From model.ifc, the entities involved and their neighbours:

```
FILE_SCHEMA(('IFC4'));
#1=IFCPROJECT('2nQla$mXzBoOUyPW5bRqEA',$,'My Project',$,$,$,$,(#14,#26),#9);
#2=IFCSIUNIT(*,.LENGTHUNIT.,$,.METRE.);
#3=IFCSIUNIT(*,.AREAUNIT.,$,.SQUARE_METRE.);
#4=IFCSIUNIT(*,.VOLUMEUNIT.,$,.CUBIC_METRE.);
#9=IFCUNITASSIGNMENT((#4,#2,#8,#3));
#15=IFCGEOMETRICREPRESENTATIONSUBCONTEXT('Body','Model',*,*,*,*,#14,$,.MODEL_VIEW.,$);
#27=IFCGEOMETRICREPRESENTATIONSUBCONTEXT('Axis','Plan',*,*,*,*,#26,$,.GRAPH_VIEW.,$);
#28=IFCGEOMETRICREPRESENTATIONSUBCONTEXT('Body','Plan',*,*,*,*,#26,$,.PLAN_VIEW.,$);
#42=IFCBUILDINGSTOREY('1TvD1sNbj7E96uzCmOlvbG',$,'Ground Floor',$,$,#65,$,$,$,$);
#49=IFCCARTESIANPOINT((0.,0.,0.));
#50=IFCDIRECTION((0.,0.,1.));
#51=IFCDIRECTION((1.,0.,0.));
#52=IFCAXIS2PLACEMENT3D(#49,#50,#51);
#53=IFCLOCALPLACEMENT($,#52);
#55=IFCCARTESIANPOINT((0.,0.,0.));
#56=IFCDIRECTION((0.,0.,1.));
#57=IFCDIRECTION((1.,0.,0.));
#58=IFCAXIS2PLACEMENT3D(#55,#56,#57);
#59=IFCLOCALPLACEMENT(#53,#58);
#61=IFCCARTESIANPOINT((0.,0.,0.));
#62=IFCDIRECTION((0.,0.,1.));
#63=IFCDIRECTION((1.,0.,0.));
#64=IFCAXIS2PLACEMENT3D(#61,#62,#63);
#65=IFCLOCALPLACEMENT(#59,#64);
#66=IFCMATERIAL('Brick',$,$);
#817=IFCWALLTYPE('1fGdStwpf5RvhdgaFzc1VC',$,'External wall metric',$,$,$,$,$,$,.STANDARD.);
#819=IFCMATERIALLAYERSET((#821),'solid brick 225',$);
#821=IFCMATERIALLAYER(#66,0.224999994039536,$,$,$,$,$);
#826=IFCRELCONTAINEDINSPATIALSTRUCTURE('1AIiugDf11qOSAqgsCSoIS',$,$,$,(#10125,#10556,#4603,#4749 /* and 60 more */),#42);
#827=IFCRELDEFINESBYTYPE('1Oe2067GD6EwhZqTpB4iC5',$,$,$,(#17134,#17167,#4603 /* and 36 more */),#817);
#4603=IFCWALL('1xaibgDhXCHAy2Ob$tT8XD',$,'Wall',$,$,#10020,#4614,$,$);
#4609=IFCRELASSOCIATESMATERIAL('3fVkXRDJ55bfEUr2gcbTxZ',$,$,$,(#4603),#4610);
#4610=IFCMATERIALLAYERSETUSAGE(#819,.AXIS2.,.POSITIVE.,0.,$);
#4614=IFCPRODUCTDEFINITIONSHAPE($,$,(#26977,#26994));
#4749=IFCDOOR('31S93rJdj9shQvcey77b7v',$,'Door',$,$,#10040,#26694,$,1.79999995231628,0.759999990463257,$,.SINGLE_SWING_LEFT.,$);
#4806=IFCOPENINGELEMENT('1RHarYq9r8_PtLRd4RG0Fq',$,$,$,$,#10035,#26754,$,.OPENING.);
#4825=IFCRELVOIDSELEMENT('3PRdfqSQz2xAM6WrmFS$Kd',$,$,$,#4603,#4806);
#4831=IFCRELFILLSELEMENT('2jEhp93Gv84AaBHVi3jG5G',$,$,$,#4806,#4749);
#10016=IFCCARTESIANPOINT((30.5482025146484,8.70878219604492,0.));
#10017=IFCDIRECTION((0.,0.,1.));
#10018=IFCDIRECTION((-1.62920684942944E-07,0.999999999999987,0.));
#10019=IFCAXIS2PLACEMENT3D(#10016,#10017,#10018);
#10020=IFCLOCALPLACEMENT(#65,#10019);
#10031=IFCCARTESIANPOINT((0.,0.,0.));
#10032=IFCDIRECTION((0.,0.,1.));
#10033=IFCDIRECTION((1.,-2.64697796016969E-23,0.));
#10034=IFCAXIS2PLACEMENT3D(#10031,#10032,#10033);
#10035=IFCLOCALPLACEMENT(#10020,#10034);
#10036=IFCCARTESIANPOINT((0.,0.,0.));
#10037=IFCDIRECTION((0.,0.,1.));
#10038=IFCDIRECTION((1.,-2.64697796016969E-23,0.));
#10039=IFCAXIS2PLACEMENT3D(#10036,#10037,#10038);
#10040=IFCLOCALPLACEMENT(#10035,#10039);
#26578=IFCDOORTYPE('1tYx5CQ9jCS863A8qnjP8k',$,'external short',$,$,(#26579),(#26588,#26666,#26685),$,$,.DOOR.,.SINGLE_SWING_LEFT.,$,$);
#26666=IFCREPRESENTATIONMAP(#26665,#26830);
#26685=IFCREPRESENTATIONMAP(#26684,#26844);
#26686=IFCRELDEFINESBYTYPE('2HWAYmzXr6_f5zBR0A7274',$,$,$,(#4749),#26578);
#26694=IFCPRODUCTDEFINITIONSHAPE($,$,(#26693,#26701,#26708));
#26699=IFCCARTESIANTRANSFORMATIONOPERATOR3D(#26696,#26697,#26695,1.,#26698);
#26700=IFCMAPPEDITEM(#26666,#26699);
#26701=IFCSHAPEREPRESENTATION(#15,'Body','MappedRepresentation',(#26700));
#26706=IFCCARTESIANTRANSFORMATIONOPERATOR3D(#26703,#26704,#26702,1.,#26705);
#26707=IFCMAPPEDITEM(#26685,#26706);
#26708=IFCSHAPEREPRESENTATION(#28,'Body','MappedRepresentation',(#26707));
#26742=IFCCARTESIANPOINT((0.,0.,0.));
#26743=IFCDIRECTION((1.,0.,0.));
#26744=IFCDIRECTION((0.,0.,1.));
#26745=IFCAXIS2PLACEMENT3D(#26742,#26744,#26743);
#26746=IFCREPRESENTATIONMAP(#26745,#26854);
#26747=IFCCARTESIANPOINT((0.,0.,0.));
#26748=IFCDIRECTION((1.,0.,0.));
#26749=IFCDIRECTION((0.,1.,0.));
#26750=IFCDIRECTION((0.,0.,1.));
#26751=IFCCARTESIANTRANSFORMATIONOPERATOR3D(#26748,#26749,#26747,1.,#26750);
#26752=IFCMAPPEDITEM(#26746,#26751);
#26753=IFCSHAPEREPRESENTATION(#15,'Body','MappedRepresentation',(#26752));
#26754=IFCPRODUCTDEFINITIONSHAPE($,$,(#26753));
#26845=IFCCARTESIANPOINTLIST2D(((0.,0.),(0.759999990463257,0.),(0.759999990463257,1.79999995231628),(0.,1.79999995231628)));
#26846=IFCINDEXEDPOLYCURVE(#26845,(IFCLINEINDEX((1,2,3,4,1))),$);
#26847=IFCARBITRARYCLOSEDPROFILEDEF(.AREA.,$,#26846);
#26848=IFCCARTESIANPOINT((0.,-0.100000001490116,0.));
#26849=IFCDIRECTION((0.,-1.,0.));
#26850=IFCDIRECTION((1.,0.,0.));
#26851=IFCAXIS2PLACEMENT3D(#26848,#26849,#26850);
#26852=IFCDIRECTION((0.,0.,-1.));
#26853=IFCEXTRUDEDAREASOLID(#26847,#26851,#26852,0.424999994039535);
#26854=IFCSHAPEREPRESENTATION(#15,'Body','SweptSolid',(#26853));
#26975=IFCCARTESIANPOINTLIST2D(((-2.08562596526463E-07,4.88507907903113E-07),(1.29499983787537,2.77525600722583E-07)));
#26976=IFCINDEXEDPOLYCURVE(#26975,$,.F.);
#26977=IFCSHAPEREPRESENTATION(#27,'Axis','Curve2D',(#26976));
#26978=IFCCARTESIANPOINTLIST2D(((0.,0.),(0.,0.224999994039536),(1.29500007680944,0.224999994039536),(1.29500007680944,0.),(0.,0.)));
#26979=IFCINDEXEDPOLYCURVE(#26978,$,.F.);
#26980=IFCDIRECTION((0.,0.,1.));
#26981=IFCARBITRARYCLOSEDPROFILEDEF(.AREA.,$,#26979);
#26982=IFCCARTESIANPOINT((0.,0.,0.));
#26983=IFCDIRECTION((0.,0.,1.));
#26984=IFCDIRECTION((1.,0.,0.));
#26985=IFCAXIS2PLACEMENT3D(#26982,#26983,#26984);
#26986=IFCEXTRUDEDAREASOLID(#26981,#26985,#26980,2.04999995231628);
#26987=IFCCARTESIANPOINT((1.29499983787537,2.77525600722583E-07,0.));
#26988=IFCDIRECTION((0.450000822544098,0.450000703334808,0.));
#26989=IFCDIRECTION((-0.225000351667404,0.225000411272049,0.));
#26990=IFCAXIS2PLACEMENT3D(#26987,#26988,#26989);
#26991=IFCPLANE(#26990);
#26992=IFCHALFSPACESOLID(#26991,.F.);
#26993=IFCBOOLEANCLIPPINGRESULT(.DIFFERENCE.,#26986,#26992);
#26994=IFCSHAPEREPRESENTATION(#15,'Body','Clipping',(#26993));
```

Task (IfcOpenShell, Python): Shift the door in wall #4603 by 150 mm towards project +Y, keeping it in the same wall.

```python
import ifcopenshell
import ifcopenshell.api.geometry
import ifcopenshell.util.placement

model = ifcopenshell.open("model.ifc")

door = model.by_guid("31S93rJdj9shQvcey77b7v")
opening = door.FillsVoids[0].RelatingOpeningElement
wall = opening.VoidsElements[0].RelatingBuildingElement

wall_matrix = ifcopenshell.util.placement.get_local_placement(wall.ObjectPlacement)
shift = wall_matrix[:3, 0] * 0.15
before = ifcopenshell.util.placement.get_local_placement(door.ObjectPlacement)[:3, 3].copy()

# The door is placed relative to its opening, so it follows when the opening moves.
matrix = ifcopenshell.util.placement.get_local_placement(opening.ObjectPlacement)
matrix[:3, 3] += shift
ifcopenshell.api.geometry.edit_object_placement(
    model, product=opening, matrix=matrix, is_si=False, should_transform_children=True
)

after = ifcopenshell.util.placement.get_local_placement(door.ObjectPlacement)[:3, 3]
print("door moved by", (after - before).round(3) + 0.0)

model.write("model_updated.ifc")
```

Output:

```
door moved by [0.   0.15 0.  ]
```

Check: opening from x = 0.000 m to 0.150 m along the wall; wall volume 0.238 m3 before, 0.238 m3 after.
